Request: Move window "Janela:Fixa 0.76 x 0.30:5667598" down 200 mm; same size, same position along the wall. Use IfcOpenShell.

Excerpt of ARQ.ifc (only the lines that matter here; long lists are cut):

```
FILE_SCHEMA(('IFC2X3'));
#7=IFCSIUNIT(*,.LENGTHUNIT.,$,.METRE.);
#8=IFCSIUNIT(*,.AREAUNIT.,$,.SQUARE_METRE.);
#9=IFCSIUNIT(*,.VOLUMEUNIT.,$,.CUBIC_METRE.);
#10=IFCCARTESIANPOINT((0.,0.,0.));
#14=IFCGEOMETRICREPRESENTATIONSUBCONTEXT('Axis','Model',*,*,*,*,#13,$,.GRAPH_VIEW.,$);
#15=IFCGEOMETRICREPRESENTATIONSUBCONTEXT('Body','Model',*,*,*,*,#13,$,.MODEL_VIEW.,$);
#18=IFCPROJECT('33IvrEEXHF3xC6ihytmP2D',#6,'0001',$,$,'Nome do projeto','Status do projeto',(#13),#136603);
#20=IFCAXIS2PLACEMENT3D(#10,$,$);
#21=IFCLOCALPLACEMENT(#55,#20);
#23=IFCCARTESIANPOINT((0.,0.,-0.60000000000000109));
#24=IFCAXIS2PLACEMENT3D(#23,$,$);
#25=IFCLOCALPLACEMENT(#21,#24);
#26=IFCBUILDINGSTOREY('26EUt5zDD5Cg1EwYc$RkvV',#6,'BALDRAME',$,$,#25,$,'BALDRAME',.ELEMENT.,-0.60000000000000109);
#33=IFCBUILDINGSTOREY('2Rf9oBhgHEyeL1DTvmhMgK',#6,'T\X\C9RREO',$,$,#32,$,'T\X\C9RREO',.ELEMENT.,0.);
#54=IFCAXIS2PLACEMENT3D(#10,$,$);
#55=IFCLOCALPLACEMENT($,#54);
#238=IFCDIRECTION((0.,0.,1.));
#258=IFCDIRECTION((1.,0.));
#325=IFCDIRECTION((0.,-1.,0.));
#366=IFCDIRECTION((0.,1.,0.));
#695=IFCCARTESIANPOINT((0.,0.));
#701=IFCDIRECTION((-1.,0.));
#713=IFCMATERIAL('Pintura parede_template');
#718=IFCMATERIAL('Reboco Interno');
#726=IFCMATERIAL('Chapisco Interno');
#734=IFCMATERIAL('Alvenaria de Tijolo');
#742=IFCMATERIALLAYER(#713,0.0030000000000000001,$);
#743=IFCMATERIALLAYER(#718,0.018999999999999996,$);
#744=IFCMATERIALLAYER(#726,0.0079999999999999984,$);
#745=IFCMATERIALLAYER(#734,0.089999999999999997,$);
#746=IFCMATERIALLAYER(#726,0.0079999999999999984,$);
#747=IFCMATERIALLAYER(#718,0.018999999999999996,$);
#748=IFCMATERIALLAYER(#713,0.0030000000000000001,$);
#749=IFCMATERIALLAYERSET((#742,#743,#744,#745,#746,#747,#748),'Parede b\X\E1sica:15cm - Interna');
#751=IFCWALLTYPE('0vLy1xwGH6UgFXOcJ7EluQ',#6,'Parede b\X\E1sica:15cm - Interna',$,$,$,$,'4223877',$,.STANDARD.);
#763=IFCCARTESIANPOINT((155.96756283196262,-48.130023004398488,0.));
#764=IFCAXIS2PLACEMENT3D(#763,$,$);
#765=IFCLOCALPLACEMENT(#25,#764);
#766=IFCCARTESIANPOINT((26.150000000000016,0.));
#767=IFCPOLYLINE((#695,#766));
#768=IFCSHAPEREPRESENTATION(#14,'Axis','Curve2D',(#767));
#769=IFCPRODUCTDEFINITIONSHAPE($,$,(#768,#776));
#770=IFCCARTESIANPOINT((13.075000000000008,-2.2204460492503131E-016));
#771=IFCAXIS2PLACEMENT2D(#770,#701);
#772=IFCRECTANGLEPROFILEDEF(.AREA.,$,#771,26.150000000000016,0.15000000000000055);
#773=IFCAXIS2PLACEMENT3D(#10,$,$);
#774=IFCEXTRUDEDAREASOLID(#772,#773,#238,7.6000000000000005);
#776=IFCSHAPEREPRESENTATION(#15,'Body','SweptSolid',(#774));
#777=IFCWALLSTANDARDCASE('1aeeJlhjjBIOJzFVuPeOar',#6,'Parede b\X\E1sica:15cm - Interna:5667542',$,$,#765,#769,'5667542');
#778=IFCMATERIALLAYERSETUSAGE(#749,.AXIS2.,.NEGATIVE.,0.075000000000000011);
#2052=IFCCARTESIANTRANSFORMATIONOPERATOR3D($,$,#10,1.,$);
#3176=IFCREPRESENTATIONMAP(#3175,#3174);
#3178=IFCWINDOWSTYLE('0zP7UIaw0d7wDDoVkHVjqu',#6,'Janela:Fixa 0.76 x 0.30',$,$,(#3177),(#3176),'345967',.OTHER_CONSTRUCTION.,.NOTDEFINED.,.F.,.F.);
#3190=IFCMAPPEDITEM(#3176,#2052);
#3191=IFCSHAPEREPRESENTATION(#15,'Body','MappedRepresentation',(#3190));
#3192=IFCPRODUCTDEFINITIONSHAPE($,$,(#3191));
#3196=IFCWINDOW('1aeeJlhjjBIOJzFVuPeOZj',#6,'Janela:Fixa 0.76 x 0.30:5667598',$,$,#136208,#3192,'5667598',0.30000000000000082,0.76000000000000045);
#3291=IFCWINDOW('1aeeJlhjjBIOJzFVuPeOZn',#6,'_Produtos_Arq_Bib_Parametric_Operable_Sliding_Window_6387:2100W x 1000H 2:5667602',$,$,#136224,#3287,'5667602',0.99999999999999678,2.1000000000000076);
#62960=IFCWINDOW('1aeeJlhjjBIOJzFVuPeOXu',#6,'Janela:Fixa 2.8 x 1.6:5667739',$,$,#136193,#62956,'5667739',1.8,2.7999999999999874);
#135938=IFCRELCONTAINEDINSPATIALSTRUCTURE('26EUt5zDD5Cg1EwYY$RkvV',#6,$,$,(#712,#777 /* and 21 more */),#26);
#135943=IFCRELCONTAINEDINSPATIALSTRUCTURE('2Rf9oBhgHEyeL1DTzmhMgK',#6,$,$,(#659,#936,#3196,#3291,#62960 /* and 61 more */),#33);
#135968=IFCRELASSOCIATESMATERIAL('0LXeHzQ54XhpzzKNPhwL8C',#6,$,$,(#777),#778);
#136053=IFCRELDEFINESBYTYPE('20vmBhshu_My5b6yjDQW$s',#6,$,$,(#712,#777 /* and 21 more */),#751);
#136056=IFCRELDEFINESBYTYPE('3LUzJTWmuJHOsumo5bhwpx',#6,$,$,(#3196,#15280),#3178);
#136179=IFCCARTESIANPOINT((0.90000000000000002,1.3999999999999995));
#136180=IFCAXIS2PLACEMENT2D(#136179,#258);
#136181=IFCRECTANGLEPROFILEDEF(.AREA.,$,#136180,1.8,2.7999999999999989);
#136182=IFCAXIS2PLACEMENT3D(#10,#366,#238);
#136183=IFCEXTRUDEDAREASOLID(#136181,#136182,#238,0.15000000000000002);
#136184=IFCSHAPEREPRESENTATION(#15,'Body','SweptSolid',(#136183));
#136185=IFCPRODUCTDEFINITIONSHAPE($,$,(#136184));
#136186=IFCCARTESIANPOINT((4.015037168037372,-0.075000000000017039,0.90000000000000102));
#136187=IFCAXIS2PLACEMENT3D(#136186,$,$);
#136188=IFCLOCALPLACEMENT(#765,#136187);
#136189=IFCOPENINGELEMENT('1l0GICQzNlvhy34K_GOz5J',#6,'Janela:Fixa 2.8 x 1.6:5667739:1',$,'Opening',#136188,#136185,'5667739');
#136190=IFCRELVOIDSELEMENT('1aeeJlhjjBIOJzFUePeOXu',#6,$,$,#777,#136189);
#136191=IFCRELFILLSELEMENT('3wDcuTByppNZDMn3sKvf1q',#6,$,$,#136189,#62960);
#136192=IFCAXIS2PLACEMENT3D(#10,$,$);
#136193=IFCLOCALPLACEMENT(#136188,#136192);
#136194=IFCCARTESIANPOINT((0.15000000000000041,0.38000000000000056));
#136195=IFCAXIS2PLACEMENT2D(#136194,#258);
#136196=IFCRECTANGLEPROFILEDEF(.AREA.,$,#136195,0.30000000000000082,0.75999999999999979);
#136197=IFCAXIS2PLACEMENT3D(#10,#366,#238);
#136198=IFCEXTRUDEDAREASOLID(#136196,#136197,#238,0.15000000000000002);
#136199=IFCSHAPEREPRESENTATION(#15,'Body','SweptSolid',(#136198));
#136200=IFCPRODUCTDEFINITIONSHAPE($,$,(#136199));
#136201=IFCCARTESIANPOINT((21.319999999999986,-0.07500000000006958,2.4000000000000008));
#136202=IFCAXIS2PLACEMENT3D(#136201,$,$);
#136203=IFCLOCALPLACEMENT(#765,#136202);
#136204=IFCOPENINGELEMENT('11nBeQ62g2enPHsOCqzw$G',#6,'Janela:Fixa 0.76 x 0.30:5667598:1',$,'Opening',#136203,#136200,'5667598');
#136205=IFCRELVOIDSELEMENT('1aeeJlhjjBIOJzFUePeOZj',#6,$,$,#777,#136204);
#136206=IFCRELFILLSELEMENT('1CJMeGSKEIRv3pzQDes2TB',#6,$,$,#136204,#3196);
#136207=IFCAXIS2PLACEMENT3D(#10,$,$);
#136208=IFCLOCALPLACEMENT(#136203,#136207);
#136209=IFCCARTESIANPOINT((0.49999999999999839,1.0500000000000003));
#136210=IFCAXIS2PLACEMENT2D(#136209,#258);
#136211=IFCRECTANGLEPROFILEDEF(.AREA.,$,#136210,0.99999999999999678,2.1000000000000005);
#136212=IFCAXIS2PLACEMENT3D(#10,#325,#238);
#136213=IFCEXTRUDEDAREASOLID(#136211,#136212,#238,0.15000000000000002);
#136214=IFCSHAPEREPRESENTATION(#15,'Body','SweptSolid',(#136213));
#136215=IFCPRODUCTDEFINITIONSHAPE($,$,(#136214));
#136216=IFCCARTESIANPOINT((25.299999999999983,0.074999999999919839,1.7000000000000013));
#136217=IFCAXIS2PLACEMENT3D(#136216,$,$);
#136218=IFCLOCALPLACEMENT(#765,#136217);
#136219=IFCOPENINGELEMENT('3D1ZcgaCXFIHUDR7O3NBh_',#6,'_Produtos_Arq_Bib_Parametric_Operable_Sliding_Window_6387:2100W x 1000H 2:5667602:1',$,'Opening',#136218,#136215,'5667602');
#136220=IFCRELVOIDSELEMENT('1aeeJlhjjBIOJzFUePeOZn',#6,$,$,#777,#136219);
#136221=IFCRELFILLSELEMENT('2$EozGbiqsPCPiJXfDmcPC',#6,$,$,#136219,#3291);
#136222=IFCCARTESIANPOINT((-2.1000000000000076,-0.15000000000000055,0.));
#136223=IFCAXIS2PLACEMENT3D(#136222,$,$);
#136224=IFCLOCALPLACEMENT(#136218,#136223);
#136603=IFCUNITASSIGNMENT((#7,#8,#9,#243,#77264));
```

```python
import numpy as np
import ifcopenshell
import ifcopenshell.api.geometry
import ifcopenshell.util.placement
import ifcopenshell.util.unit

model = ifcopenshell.open("ARQ.ifc")
unit_scale = ifcopenshell.util.unit.calculate_unit_scale(model)

window = model.by_id(3196)
opening = window.FillsVoids[0].RelatingOpeningElement
dz = -0.2

shift = np.array([0.0, 0.0, dz])
# The window is placed relative to its opening, so it follows when the opening moves.
matrix = ifcopenshell.util.placement.get_local_placement(opening.ObjectPlacement)
matrix[:3, 3] += shift
ifcopenshell.api.geometry.edit_object_placement(
    model, product=opening, matrix=matrix, is_si=False, should_transform_children=True
)

print(f"moved by {dz * unit_scale:+.3f} m")

model.write("ARQ_updated.ifc")
```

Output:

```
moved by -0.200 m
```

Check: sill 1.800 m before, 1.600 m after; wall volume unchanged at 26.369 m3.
